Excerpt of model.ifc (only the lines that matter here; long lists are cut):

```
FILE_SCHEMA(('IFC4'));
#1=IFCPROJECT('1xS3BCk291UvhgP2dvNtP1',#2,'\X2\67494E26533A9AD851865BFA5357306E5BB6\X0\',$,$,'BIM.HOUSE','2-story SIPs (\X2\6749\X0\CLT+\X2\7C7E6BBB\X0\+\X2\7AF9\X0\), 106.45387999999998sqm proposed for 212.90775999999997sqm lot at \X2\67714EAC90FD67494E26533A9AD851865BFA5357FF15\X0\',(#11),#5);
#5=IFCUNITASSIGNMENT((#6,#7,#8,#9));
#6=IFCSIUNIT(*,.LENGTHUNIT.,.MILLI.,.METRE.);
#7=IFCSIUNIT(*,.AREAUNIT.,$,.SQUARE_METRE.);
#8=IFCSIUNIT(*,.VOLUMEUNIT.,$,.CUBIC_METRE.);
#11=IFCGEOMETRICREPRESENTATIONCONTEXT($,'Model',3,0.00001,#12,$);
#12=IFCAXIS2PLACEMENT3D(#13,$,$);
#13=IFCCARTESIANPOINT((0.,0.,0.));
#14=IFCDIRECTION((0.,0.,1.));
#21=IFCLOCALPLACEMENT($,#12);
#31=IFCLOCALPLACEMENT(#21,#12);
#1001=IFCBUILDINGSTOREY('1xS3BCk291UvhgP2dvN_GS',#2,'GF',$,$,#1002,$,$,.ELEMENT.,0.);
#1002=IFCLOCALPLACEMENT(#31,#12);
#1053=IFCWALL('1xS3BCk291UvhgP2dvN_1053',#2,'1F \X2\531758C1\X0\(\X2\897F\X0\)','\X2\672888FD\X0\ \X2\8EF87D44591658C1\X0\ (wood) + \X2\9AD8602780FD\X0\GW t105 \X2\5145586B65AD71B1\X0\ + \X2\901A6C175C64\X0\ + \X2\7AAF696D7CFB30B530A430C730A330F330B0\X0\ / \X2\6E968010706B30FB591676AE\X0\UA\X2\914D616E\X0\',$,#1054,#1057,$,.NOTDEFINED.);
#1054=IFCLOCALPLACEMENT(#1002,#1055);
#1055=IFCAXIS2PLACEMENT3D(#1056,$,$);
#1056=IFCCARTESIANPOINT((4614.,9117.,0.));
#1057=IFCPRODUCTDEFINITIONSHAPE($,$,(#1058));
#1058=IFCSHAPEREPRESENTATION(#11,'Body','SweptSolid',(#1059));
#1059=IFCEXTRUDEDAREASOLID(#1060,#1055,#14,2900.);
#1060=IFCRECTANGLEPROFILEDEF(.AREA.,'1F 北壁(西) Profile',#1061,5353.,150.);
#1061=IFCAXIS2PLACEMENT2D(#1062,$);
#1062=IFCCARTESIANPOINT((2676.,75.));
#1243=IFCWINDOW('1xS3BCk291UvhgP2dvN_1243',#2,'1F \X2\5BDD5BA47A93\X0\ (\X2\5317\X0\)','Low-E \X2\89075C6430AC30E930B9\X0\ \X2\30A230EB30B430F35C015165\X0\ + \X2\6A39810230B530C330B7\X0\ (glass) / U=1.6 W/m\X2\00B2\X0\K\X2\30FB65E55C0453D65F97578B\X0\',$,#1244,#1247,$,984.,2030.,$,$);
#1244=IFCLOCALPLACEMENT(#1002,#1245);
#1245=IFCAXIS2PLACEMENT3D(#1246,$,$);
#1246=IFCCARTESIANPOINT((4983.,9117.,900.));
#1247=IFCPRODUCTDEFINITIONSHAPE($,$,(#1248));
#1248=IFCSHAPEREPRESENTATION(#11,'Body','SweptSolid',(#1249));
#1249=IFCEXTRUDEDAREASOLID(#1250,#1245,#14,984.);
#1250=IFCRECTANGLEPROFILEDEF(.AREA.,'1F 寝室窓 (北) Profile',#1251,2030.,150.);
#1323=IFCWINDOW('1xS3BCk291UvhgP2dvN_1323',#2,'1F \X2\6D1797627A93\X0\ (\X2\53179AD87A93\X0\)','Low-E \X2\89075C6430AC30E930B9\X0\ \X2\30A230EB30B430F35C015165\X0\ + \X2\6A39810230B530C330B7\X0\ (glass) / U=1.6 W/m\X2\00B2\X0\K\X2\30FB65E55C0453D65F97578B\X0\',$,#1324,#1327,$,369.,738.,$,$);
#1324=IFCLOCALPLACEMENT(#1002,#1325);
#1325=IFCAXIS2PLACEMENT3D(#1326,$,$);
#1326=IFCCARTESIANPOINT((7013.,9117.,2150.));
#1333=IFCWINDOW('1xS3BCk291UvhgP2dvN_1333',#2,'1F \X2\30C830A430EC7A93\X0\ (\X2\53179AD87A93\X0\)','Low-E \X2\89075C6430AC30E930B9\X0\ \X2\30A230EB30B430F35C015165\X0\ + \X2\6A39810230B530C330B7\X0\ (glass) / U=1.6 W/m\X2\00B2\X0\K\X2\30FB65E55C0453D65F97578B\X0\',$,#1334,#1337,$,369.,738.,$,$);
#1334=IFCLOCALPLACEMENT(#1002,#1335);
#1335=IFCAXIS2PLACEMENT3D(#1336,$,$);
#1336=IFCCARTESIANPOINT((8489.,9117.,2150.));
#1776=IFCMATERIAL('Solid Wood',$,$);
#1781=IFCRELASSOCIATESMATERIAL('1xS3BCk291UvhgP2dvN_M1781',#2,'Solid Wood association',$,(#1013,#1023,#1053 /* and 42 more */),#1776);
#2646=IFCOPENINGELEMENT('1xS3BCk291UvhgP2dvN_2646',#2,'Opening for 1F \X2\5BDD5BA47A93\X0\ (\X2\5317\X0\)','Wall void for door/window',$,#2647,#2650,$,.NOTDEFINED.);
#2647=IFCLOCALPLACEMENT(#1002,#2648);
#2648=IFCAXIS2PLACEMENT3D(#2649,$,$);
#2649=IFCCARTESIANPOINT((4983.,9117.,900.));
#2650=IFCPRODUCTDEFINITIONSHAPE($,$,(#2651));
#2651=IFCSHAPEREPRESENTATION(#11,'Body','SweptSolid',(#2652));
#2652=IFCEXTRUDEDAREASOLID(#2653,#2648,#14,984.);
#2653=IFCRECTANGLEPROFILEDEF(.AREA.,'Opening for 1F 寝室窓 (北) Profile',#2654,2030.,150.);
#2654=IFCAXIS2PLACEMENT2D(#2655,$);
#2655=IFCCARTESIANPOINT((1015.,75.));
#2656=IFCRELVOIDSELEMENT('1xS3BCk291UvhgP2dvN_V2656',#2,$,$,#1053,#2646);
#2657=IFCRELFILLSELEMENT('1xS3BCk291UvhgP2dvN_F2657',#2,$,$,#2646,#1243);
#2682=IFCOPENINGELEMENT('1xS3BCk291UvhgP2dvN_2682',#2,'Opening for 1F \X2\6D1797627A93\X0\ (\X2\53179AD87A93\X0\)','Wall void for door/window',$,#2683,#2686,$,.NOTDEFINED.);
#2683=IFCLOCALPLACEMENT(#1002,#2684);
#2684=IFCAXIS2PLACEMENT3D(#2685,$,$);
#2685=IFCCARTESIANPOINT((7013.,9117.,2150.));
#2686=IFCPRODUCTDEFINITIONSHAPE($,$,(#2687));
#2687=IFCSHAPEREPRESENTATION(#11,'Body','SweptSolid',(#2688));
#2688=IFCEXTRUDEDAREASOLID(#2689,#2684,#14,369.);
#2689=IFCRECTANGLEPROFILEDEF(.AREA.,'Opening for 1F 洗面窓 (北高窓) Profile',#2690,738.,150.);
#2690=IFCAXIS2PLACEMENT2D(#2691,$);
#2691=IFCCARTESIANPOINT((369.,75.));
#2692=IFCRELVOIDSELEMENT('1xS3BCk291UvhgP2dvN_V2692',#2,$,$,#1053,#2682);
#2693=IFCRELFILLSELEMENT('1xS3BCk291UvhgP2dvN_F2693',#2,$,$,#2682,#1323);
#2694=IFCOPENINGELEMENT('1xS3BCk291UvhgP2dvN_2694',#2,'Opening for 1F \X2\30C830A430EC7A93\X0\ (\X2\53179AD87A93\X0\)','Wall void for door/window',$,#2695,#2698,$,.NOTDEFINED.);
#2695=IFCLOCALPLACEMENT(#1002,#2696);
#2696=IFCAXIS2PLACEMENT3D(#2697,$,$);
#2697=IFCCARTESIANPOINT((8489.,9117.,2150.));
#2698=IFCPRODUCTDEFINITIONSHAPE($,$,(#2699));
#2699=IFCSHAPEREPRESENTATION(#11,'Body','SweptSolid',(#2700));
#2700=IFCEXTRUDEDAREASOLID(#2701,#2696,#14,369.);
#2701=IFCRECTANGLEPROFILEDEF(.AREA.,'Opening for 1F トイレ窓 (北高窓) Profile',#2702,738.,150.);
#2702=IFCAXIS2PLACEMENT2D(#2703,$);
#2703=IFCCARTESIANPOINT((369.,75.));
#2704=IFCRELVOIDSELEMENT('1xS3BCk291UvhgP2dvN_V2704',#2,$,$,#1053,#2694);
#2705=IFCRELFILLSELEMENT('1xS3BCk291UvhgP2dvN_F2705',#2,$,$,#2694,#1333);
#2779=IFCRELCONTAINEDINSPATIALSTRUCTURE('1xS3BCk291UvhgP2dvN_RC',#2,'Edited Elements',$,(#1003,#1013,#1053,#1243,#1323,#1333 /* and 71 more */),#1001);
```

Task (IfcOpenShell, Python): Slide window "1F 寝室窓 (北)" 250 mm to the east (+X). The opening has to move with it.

```python
import ifcopenshell
import ifcopenshell.api.geometry
import ifcopenshell.util.placement
import ifcopenshell.util.unit

model = ifcopenshell.open("model.ifc")
unit_scale = ifcopenshell.util.unit.calculate_unit_scale(model)

window = model.by_guid("1xS3BCk291UvhgP2dvN_1243")
opening = window.FillsVoids[0].RelatingOpeningElement
wall = opening.VoidsElements[0].RelatingBuildingElement

wall_matrix = ifcopenshell.util.placement.get_local_placement(wall.ObjectPlacement)
shift = wall_matrix[:3, 0] * 0.25 / unit_scale
before = ifcopenshell.util.placement.get_local_placement(window.ObjectPlacement)[:3, 3].copy()

# The window is not placed relative to its opening, so move both.
for product in (opening, window):
    matrix = ifcopenshell.util.placement.get_local_placement(product.ObjectPlacement)
    matrix[:3, 3] += shift
    ifcopenshell.api.geometry.edit_object_placement(model, product=product, matrix=matrix, is_si=False)

after = ifcopenshell.util.placement.get_local_placement(window.ObjectPlacement)[:3, 3]
print("window moved by", (after - before).round(3) + 0.0)

model.write("model_updated.ifc")
```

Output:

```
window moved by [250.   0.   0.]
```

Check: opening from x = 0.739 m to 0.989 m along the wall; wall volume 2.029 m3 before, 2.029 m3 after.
